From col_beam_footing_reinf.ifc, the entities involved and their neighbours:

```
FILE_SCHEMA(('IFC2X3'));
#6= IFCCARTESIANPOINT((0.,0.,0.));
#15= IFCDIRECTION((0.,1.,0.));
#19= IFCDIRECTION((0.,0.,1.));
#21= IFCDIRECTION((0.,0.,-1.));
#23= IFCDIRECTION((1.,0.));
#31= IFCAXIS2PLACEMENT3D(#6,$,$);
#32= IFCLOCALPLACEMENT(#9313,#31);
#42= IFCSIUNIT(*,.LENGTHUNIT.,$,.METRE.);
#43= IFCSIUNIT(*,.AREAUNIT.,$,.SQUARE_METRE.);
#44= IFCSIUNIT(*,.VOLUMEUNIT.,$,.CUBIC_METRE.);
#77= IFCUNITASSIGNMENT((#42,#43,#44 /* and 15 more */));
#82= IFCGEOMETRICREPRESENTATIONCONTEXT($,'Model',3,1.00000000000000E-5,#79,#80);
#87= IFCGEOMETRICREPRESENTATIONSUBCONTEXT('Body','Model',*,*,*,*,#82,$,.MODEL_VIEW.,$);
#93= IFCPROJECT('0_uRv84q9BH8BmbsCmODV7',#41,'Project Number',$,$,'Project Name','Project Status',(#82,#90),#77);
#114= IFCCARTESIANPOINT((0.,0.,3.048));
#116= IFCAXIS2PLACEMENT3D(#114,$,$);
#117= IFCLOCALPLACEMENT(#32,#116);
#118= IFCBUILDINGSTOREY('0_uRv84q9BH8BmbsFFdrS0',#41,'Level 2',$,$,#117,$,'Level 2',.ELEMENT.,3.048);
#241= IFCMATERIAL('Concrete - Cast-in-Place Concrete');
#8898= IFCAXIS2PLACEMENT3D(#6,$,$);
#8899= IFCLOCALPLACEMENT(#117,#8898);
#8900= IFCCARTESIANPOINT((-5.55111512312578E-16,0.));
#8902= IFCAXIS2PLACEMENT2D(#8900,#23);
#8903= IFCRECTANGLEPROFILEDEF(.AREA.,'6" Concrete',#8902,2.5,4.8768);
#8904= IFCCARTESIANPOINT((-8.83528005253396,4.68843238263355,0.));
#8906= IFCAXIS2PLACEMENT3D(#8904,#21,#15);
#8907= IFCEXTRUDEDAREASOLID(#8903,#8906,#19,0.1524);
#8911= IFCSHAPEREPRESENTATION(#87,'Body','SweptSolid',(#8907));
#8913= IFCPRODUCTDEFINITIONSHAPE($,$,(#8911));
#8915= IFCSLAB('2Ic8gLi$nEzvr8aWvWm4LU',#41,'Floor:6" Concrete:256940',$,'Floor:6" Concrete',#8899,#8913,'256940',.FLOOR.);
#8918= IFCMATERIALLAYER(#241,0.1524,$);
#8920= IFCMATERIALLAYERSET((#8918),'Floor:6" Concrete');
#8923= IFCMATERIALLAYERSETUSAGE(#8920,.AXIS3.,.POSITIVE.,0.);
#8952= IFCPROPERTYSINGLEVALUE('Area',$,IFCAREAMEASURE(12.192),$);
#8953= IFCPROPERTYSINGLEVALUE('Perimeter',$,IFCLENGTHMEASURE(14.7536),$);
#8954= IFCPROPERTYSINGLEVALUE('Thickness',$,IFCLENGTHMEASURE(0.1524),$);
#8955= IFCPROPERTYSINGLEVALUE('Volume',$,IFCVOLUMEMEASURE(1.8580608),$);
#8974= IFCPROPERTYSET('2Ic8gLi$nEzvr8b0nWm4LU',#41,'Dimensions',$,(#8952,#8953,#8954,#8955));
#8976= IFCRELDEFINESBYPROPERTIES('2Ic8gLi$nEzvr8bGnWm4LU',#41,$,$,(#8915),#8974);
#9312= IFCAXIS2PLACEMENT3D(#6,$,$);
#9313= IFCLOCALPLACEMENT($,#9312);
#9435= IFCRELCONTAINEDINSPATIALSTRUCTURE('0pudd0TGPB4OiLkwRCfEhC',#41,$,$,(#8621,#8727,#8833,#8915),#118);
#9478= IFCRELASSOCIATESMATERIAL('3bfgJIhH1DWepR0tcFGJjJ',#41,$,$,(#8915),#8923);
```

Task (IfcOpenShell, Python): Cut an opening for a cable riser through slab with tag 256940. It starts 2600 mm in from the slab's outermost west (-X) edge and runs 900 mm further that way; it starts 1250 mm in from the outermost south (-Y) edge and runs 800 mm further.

```python
import numpy as np
import ifcopenshell
import ifcopenshell.api.feature
import ifcopenshell.api.geometry
import ifcopenshell.api.pset
import ifcopenshell.api.root
import ifcopenshell.geom
import ifcopenshell.util.element
import ifcopenshell.util.placement
import ifcopenshell.util.representation
import ifcopenshell.util.shape
import ifcopenshell.util.unit

model = ifcopenshell.open("col_beam_footing_reinf.ifc")
unit_scale = ifcopenshell.util.unit.calculate_unit_scale(model)
area_scale = ifcopenshell.util.unit.calculate_unit_scale(model, "AREAUNIT")
volume_scale = ifcopenshell.util.unit.calculate_unit_scale(model, "VOLUMEUNIT")
settings = ifcopenshell.geom.settings()


def volume(element):
    """Net volume in cubic metres, openings subtracted."""
    shape = ifcopenshell.geom.create_shape(settings, element)
    return ifcopenshell.util.shape.get_volume(shape.geometry)


slab = model.by_guid("2Ic8gLi$nEzvr8aWvWm4LU")
before = volume(slab)

# Extent in the slab's own axes, in metres. The edges named are its -X and -Y sides.
slab_shape = ifcopenshell.geom.create_shape(settings, slab)
vertices = ifcopenshell.util.shape.get_vertices(slab_shape.geometry)
x_min, y_min, bottom = vertices.min(axis=0)
top = vertices[:, 2].max()

opening = ifcopenshell.api.root.create_entity(model, ifc_class="IfcOpeningElement", name="Cable riser opening")
context = ifcopenshell.util.representation.get_context(model, "Model", "Body", "MODEL_VIEW")
width, depth = 0.9, 0.8
outline = [(0.0, 0.0), (width, 0.0), (width, depth), (0.0, depth), (0.0, 0.0)]
# Overshoot both faces by 50 mm so the cut is clean.
shape = ifcopenshell.api.geometry.add_slab_representation(
    model, context=context, depth=top - bottom + 0.1, polyline=outline
)
ifcopenshell.api.geometry.assign_representation(model, product=opening, representation=shape)

matrix = ifcopenshell.util.placement.get_local_placement(slab.ObjectPlacement)
matrix[:, 3] = matrix @ np.append(np.array([x_min + 2.6, y_min + 1.25, bottom - 0.05]) / unit_scale, 1.0)
ifcopenshell.api.geometry.edit_object_placement(model, product=opening, matrix=matrix, is_si=False)
ifcopenshell.api.feature.add_feature(model, feature=opening, element=slab)

after = volume(slab)

# Update the slab's stored quantities.
pset = model.by_id(ifcopenshell.util.element.get_pset(slab, "Dimensions", should_inherit=False)["id"])
ifcopenshell.api.pset.edit_pset(model, pset=pset, properties={
    "Area": model.create_entity("IfcAreaMeasure", after / (top - bottom) / area_scale),
    "Volume": model.create_entity("IfcVolumeMeasure", after / volume_scale),
})

print(f"slab volume {before:.3f} -> {after:.3f} m3")

model.write("col_beam_footing_reinf_updated.ifc")
```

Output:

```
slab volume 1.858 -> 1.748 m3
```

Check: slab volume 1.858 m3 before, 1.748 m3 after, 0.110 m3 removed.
